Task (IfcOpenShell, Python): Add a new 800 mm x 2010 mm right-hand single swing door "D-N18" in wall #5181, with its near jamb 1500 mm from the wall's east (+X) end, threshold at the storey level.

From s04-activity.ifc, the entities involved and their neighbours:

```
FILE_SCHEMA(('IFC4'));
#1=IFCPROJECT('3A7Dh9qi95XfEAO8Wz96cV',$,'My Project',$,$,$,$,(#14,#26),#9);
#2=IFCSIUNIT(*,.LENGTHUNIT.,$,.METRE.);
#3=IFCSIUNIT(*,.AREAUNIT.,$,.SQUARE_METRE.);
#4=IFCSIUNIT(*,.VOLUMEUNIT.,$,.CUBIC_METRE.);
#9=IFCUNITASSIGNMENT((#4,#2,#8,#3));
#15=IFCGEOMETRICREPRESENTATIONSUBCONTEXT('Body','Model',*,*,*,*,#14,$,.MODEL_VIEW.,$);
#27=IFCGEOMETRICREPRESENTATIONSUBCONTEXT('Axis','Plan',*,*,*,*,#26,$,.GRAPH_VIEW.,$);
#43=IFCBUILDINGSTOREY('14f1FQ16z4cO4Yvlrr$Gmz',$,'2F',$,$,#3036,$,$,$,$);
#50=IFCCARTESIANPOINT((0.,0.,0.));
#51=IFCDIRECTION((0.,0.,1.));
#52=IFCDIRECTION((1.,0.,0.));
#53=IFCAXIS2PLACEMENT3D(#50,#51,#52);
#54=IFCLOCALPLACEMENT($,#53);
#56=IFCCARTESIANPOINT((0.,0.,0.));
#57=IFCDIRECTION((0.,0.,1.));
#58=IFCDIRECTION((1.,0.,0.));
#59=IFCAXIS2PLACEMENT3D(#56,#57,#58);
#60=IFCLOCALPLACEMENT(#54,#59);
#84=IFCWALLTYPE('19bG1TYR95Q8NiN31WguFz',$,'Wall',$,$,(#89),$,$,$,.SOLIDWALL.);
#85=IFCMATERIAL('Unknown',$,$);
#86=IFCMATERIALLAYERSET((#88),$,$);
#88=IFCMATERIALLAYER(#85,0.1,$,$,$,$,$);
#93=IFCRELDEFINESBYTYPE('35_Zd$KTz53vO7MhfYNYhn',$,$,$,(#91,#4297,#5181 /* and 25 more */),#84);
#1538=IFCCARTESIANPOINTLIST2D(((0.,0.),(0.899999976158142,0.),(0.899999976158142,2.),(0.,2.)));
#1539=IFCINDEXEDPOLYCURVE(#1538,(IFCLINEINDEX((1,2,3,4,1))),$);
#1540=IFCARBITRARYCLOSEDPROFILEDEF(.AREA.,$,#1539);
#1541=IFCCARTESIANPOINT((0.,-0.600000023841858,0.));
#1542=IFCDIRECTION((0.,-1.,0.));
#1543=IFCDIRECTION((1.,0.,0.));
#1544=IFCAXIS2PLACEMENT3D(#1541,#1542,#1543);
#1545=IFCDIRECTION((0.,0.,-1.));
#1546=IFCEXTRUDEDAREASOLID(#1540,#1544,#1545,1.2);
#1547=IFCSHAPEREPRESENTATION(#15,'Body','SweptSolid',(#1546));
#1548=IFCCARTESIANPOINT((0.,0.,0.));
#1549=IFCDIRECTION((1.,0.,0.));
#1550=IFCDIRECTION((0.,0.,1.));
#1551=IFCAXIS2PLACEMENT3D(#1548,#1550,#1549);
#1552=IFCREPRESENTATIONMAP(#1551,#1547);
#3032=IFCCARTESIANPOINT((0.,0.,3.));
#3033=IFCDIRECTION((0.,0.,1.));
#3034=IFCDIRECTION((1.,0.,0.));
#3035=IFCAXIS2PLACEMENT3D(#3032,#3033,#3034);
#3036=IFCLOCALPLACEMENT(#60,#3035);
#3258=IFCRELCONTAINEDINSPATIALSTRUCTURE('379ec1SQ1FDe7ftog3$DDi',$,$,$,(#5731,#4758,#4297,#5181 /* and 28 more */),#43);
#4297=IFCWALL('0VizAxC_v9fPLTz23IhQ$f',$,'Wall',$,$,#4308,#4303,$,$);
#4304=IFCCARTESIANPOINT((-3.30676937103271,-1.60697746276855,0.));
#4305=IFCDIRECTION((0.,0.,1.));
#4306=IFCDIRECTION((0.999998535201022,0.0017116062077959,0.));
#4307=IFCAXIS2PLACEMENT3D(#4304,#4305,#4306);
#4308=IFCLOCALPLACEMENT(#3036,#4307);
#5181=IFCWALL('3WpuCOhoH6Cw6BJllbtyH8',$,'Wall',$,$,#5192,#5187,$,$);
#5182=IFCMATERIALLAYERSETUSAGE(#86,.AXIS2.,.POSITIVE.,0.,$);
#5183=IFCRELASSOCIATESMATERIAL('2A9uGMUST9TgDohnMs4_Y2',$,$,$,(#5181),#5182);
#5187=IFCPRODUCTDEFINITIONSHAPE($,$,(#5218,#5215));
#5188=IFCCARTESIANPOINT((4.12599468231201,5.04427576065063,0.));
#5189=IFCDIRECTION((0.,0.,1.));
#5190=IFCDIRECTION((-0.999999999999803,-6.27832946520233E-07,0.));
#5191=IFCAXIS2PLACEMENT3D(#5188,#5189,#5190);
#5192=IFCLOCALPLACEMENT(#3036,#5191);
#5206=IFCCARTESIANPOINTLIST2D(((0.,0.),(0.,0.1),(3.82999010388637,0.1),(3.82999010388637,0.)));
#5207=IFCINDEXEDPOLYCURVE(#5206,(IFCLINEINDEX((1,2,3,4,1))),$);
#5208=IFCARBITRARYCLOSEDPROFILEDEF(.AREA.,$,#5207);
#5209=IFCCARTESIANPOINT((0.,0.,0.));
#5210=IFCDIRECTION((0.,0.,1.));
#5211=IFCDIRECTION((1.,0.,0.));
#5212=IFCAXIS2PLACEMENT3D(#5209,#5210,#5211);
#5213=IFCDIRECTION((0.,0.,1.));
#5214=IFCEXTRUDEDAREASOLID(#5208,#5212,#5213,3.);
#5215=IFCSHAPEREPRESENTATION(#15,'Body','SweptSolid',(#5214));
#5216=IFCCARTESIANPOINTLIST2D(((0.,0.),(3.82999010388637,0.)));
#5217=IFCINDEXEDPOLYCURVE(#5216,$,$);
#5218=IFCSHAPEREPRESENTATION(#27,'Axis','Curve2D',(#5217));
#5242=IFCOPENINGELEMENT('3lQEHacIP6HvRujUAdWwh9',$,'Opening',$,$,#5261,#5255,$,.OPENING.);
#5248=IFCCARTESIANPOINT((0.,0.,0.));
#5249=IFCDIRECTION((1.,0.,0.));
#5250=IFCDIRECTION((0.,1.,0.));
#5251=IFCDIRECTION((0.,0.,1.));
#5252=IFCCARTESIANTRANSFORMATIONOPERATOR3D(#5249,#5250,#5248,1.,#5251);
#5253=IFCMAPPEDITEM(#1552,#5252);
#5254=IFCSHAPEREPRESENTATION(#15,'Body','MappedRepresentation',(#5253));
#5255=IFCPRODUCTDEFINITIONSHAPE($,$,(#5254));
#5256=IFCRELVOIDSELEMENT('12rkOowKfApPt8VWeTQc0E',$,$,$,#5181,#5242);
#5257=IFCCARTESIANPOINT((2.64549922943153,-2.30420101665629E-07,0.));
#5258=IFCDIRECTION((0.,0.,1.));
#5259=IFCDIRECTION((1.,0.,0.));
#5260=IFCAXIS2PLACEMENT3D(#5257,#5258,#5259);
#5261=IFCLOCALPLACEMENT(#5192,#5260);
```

```python
import numpy as np
import ifcopenshell
import ifcopenshell.api.feature
import ifcopenshell.api.geometry
import ifcopenshell.api.root
import ifcopenshell.api.spatial
import ifcopenshell.geom
import ifcopenshell.util.element
import ifcopenshell.util.placement
import ifcopenshell.util.representation
import ifcopenshell.util.shape
import ifcopenshell.util.unit

model = ifcopenshell.open("s04-activity.ifc")
unit_scale = ifcopenshell.util.unit.calculate_unit_scale(model)
settings = ifcopenshell.geom.settings()


def volume(element):
    """Net volume in cubic metres, openings subtracted."""
    shape = ifcopenshell.geom.create_shape(settings, element)
    return ifcopenshell.util.shape.get_volume(shape.geometry)


wall = model.by_id(5181)
storey = ifcopenshell.util.element.get_container(wall, ifc_class="IfcBuildingStorey")
context = ifcopenshell.util.representation.get_context(model, "Model", "Body", "MODEL_VIEW")
before = volume(wall)

width, height, from_end, sill = 0.8, 2.01, 1.5, 0.0  # metres

# The wall runs along its own X axis, and the end named is its -X end.
wall_shape = ifcopenshell.geom.create_shape(settings, wall)
x, y, z = ifcopenshell.util.shape.get_vertices(wall_shape.geometry).T
start = x.min() + from_end
face, thickness = float(y.min()), float(y.max() - y.min())
wall_matrix = ifcopenshell.util.placement.get_local_placement(wall.ObjectPlacement)
level = ifcopenshell.util.placement.get_local_placement(storey.ObjectPlacement)[2, 3]


def in_wall(x, y):
    """Placement at x, y metres in the wall's axes, at sill height."""
    matrix = wall_matrix.copy()
    matrix[:, 3] = wall_matrix @ np.array([x / unit_scale, y / unit_scale, 0.0, 1.0])
    matrix[2, 3] = level + sill / unit_scale
    return matrix


# Opening: a box that overshoots both wall faces by 50 mm.
opening = ifcopenshell.api.root.create_entity(model, ifc_class="IfcOpeningElement", predefined_type="OPENING")
box = ifcopenshell.api.geometry.add_wall_representation(
    model, context=context, length=width, height=height, thickness=thickness + 0.1
)
ifcopenshell.api.geometry.assign_representation(model, product=opening, representation=box)
ifcopenshell.api.geometry.edit_object_placement(model, product=opening, matrix=in_wall(start, face - 0.05), is_si=False)
ifcopenshell.api.feature.add_feature(model, feature=opening, element=wall)

door = ifcopenshell.api.root.create_entity(model, ifc_class="IfcDoor", name="D-N18", predefined_type="DOOR")
door.OverallWidth, door.OverallHeight = width / unit_scale, height / unit_scale
door.OperationType = "SINGLE_SWING_RIGHT"
body = ifcopenshell.api.geometry.add_door_representation(
    model,
    context=context,
    overall_width=door.OverallWidth,
    overall_height=door.OverallHeight,
    operation_type="SINGLE_SWING_RIGHT",
    lining_properties={"LiningDepth": thickness / unit_scale, "ThresholdDepth": thickness / unit_scale},
)
ifcopenshell.api.geometry.assign_representation(model, product=door, representation=body)
ifcopenshell.api.spatial.assign_container(model, products=[door], relating_structure=storey)
ifcopenshell.api.feature.add_filling(model, opening=opening, element=door)

# The lining spans the wall, so the door starts at the wall face.
ifcopenshell.api.geometry.edit_object_placement(model, product=door, matrix=in_wall(start, face), is_si=False)

after = volume(wall)

print(f"wall volume {before:.3f} -> {after:.3f} m3")

model.write("s04-activity_updated.ifc")
```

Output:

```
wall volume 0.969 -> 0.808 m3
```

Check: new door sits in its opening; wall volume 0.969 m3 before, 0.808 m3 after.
